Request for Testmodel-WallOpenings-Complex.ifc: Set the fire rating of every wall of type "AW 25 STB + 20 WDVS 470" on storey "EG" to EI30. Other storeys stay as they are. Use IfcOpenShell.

First a look at what the model holds.

```python
import ifcopenshell
import ifcopenshell.util.element

model = ifcopenshell.open("Testmodel-WallOpenings-Complex.ifc")
print(model.schema)
storey = next(s for s in model.by_type("IfcBuildingStorey") if s.Name == "EG")
walls = [e for e in ifcopenshell.util.element.get_decomposition(storey) if e.is_a("IfcWall")]
seen = {}
for e in walls:
    element_type = ifcopenshell.util.element.get_type(e)
    key = (element_type.Name if element_type != e and element_type else None, ifcopenshell.util.element.get_pset(e, "Pset_WallCommon", "FireRating"))
    seen[key] = seen.get(key, 0) + 1
for (name, value), count in sorted(seen.items(), key=str):
    print(count, "x", name, "|", value)
```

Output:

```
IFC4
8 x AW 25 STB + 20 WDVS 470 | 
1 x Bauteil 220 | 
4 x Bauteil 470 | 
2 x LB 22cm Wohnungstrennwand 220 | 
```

```python
import ifcopenshell
import ifcopenshell.api.pset
import ifcopenshell.util.element

model = ifcopenshell.open("Testmodel-WallOpenings-Complex.ifc")

storey = next(s for s in model.by_type("IfcBuildingStorey") if s.Name == "EG")
walls = [e for e in ifcopenshell.util.element.get_decomposition(storey) if e.is_a("IfcWall")]

count = 0
for e in walls:
    element_type = ifcopenshell.util.element.get_type(e)
    if element_type in (None, e) or element_type.Name != "AW 25 STB + 20 WDVS 470":
        continue
    # add_pset returns the element's existing set when there is one.
    pset = ifcopenshell.api.pset.add_pset(model, product=e, name="Pset_WallCommon")
    ifcopenshell.api.pset.edit_pset(model, pset=pset, properties={"FireRating": "EI30"})
    count += 1

print(count, "walls updated")

model.write("Testmodel-WallOpenings-Complex_edited.ifc")
```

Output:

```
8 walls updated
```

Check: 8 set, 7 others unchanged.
